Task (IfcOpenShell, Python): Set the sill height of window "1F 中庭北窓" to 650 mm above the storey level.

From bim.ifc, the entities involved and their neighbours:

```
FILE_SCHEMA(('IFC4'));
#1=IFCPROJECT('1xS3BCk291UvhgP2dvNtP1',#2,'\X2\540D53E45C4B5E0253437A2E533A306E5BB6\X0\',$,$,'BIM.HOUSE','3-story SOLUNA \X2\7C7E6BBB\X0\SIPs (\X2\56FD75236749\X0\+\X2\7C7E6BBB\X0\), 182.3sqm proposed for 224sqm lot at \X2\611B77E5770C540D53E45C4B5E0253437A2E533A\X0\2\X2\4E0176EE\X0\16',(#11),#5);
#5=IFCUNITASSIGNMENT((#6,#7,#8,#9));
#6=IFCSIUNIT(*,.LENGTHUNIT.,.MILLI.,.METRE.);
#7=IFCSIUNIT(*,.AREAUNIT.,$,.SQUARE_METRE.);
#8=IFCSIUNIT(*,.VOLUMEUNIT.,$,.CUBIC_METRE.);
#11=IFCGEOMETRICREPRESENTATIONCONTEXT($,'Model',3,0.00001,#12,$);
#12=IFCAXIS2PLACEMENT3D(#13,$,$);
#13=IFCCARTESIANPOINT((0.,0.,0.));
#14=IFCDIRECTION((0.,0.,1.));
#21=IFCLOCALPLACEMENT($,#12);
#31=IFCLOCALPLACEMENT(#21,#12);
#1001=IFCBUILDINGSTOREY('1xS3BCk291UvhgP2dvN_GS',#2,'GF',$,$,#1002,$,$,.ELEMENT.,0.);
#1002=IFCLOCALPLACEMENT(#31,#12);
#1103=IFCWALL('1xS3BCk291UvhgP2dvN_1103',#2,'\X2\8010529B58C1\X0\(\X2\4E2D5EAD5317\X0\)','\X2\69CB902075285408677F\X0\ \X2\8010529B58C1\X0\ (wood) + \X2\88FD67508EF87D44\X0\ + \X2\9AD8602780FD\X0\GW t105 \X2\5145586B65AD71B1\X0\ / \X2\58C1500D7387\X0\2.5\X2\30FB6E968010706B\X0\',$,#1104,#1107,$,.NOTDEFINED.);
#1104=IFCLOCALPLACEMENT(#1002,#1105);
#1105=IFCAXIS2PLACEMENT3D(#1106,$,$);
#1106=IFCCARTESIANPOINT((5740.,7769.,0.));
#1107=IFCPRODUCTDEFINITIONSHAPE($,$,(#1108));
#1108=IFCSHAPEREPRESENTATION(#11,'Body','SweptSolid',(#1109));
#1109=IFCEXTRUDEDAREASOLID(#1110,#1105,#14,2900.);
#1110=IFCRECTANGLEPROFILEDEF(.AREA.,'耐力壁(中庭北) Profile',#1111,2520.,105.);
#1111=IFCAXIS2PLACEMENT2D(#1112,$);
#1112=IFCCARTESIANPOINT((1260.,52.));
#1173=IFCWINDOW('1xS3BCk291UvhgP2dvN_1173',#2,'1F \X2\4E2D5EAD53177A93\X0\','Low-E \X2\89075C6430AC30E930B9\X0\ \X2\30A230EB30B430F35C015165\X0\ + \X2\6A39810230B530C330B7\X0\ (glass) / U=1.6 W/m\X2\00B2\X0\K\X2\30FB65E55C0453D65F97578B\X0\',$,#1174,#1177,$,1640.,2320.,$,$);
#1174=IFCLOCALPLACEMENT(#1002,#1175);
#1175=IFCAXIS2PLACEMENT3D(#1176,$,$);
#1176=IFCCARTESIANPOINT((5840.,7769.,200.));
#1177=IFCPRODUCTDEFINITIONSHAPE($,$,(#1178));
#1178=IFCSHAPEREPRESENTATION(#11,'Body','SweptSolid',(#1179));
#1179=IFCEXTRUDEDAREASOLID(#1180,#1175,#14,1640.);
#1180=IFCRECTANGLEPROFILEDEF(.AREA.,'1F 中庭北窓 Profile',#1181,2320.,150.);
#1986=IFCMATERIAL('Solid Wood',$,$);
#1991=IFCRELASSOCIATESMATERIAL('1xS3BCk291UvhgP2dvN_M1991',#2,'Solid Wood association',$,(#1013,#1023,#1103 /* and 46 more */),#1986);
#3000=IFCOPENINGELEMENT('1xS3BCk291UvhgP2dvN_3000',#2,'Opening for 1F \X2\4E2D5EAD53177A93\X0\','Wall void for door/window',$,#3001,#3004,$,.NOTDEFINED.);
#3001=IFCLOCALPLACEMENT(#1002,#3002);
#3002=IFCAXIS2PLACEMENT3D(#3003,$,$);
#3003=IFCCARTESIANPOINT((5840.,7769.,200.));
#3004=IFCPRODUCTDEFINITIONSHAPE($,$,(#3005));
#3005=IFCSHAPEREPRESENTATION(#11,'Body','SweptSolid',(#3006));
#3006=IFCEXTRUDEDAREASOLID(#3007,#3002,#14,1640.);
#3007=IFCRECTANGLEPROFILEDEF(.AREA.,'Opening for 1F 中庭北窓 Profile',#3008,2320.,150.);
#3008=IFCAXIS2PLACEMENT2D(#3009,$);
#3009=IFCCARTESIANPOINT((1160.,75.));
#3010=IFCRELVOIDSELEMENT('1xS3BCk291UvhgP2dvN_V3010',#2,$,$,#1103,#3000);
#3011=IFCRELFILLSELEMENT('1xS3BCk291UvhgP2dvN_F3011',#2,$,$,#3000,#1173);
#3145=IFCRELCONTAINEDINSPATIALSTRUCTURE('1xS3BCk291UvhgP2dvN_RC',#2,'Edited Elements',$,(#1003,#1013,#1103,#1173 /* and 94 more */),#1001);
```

```python
import numpy as np
import ifcopenshell
import ifcopenshell.api.geometry
import ifcopenshell.geom
import ifcopenshell.util.element
import ifcopenshell.util.placement
import ifcopenshell.util.shape
import ifcopenshell.util.unit

model = ifcopenshell.open("bim.ifc")
unit_scale = ifcopenshell.util.unit.calculate_unit_scale(model)

window = model.by_guid("1xS3BCk291UvhgP2dvN_1173")
opening = window.FillsVoids[0].RelatingOpeningElement
storey = ifcopenshell.util.element.get_container(window, ifc_class="IfcBuildingStorey")
level = ifcopenshell.util.placement.get_local_placement(storey.ObjectPlacement)[2, 3]

# The opening's origin need not be at the sill, so measure its lowest point.
shape = ifcopenshell.geom.create_shape(ifcopenshell.geom.settings(), opening)
bottom = ifcopenshell.util.shape.get_shape_bottom_elevation(shape, shape.geometry) / unit_scale
dz = level + 650.0 - bottom

shift = np.array([0.0, 0.0, dz])
# The window is not placed relative to its opening, so move both.
for product in (opening, window):
    matrix = ifcopenshell.util.placement.get_local_placement(product.ObjectPlacement)
    matrix[:3, 3] += shift
    ifcopenshell.api.geometry.edit_object_placement(model, product=product, matrix=matrix, is_si=False)

print(f"moved by {dz * unit_scale:+.3f} m")

model.write("bim_edited.ifc")
```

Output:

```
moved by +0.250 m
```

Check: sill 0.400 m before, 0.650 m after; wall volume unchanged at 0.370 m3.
